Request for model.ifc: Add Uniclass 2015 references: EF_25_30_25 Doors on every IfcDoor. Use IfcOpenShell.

First a look at what the model holds.

```python
import ifcopenshell

model = ifcopenshell.open("model.ifc")
print(model.schema)
print("classifications:", [c.Name for c in model.by_type("IfcClassification")])
for ifc_class in ("IfcDoor", "IfcRoof", "IfcStair", "IfcWall", "IfcWindow"):
    print(ifc_class, len(model.by_type(ifc_class)))
```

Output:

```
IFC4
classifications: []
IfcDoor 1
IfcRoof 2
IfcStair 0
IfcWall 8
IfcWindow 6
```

```python
import ifcopenshell
import ifcopenshell.api.classification

model = ifcopenshell.open("model.ifc")

system = ifcopenshell.api.classification.add_classification(model, classification="Uniclass 2015")

codes = {
    "IfcDoor": ("EF_25_30_25", "Doors"),
}
for ifc_class, (code, name) in codes.items():
    products = model.by_type(ifc_class)
    ifcopenshell.api.classification.add_reference(
        model, products=products, classification=system, identification=code, name=name
    )
    print(code, len(products))

model.write("model_updated.ifc")
```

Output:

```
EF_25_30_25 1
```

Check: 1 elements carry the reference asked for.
